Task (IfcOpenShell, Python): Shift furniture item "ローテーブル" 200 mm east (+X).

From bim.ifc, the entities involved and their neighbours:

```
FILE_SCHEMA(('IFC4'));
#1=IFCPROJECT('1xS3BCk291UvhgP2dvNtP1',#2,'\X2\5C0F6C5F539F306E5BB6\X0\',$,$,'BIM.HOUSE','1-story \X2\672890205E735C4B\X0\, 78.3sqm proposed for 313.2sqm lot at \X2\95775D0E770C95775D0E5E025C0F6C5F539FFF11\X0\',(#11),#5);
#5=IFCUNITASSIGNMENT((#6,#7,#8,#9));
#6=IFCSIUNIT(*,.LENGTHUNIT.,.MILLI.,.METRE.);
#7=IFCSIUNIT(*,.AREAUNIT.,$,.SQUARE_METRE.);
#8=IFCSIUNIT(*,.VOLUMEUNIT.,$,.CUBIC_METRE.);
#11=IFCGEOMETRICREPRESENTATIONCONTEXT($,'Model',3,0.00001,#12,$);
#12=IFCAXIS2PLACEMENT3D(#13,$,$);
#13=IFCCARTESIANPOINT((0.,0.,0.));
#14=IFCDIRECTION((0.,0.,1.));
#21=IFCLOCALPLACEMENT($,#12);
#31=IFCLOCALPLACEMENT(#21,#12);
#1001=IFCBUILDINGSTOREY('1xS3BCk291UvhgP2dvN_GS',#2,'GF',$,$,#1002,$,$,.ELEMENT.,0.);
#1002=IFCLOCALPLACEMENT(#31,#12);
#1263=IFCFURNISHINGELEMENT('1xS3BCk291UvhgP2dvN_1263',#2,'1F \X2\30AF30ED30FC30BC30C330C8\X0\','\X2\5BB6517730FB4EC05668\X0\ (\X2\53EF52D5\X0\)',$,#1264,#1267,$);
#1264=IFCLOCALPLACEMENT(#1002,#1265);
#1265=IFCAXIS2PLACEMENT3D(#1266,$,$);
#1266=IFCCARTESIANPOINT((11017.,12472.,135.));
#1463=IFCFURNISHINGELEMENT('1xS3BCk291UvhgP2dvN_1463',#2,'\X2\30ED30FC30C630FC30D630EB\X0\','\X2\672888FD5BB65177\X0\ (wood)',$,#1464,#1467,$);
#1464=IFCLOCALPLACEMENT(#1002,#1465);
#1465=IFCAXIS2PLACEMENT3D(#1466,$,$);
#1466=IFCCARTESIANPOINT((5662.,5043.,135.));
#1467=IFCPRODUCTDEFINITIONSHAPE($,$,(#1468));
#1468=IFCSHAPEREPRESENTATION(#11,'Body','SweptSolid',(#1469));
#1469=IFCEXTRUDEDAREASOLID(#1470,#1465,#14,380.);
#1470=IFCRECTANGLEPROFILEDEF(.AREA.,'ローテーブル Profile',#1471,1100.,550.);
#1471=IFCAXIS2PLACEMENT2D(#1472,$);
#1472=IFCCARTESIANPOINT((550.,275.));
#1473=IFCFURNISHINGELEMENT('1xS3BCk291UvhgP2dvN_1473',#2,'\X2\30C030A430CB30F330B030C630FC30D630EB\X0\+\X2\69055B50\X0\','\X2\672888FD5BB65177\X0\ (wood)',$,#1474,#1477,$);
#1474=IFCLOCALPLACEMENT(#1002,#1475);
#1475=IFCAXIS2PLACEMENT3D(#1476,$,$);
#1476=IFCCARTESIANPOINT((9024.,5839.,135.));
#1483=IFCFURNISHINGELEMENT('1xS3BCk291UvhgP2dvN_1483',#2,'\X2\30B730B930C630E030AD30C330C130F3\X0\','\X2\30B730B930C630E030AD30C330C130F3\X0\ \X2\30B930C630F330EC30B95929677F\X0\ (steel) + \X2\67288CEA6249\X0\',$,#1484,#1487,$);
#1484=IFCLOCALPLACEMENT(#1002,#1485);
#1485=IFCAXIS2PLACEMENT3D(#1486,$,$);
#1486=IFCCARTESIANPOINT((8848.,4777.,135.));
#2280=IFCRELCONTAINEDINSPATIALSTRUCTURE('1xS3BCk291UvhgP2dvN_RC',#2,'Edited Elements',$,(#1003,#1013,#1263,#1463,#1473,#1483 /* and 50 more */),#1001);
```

```python
import ifcopenshell
import ifcopenshell.api.geometry
import ifcopenshell.util.placement
import ifcopenshell.util.unit

model = ifcopenshell.open("bim.ifc")
unit_scale = ifcopenshell.util.unit.calculate_unit_scale(model)

item = model.by_id(1463)
matrix = ifcopenshell.util.placement.get_local_placement(item.ObjectPlacement)
matrix[0, 3] += 0.2 / unit_scale
ifcopenshell.api.geometry.edit_object_placement(model, product=item, matrix=matrix, is_si=False)

print(ifcopenshell.util.placement.get_local_placement(item.ObjectPlacement).round(3) + 0.0)

model.write("bim_updated.ifc")
```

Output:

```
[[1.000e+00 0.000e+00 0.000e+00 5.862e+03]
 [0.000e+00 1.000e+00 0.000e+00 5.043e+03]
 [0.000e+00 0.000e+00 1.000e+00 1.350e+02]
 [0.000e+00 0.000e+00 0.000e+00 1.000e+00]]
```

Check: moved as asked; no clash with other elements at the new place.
